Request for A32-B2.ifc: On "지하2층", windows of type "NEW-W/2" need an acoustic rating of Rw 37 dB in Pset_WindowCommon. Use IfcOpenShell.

First a look at what the model holds.

```python
import ifcopenshell
import ifcopenshell.util.element

model = ifcopenshell.open("A32-B2.ifc")
print(model.schema)
storey = next(s for s in model.by_type("IfcBuildingStorey") if s.Name == "지하2층")
windows = [e for e in ifcopenshell.util.element.get_decomposition(storey) if e.is_a("IfcWindow")]
seen = {}
for e in windows:
    element_type = ifcopenshell.util.element.get_type(e)
    key = (element_type.Name if element_type != e and element_type else None, ifcopenshell.util.element.get_pset(e, "Pset_WindowCommon", "AcousticRating"))
    seen[key] = seen.get(key, 0) + 1
for (name, value), count in sorted(seen.items(), key=str):
    print(count, "x", name, "|", value)
```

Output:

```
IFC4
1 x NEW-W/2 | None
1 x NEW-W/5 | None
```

```python
import ifcopenshell
import ifcopenshell.api.pset
import ifcopenshell.util.element

model = ifcopenshell.open("A32-B2.ifc")

storey = next(s for s in model.by_type("IfcBuildingStorey") if s.Name == "지하2층")
windows = [e for e in ifcopenshell.util.element.get_decomposition(storey) if e.is_a("IfcWindow")]

count = 0
for e in windows:
    element_type = ifcopenshell.util.element.get_type(e)
    if element_type in (None, e) or element_type.Name != "NEW-W/2":
        continue
    # add_pset returns the element's existing set when there is one.
    pset = ifcopenshell.api.pset.add_pset(model, product=e, name="Pset_WindowCommon")
    ifcopenshell.api.pset.edit_pset(model, pset=pset, properties={"AcousticRating": "Rw 37 dB"})
    count += 1

print(count, "windows updated")

model.write("A32-B2_v2.ifc")
```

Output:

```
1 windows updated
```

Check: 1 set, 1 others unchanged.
